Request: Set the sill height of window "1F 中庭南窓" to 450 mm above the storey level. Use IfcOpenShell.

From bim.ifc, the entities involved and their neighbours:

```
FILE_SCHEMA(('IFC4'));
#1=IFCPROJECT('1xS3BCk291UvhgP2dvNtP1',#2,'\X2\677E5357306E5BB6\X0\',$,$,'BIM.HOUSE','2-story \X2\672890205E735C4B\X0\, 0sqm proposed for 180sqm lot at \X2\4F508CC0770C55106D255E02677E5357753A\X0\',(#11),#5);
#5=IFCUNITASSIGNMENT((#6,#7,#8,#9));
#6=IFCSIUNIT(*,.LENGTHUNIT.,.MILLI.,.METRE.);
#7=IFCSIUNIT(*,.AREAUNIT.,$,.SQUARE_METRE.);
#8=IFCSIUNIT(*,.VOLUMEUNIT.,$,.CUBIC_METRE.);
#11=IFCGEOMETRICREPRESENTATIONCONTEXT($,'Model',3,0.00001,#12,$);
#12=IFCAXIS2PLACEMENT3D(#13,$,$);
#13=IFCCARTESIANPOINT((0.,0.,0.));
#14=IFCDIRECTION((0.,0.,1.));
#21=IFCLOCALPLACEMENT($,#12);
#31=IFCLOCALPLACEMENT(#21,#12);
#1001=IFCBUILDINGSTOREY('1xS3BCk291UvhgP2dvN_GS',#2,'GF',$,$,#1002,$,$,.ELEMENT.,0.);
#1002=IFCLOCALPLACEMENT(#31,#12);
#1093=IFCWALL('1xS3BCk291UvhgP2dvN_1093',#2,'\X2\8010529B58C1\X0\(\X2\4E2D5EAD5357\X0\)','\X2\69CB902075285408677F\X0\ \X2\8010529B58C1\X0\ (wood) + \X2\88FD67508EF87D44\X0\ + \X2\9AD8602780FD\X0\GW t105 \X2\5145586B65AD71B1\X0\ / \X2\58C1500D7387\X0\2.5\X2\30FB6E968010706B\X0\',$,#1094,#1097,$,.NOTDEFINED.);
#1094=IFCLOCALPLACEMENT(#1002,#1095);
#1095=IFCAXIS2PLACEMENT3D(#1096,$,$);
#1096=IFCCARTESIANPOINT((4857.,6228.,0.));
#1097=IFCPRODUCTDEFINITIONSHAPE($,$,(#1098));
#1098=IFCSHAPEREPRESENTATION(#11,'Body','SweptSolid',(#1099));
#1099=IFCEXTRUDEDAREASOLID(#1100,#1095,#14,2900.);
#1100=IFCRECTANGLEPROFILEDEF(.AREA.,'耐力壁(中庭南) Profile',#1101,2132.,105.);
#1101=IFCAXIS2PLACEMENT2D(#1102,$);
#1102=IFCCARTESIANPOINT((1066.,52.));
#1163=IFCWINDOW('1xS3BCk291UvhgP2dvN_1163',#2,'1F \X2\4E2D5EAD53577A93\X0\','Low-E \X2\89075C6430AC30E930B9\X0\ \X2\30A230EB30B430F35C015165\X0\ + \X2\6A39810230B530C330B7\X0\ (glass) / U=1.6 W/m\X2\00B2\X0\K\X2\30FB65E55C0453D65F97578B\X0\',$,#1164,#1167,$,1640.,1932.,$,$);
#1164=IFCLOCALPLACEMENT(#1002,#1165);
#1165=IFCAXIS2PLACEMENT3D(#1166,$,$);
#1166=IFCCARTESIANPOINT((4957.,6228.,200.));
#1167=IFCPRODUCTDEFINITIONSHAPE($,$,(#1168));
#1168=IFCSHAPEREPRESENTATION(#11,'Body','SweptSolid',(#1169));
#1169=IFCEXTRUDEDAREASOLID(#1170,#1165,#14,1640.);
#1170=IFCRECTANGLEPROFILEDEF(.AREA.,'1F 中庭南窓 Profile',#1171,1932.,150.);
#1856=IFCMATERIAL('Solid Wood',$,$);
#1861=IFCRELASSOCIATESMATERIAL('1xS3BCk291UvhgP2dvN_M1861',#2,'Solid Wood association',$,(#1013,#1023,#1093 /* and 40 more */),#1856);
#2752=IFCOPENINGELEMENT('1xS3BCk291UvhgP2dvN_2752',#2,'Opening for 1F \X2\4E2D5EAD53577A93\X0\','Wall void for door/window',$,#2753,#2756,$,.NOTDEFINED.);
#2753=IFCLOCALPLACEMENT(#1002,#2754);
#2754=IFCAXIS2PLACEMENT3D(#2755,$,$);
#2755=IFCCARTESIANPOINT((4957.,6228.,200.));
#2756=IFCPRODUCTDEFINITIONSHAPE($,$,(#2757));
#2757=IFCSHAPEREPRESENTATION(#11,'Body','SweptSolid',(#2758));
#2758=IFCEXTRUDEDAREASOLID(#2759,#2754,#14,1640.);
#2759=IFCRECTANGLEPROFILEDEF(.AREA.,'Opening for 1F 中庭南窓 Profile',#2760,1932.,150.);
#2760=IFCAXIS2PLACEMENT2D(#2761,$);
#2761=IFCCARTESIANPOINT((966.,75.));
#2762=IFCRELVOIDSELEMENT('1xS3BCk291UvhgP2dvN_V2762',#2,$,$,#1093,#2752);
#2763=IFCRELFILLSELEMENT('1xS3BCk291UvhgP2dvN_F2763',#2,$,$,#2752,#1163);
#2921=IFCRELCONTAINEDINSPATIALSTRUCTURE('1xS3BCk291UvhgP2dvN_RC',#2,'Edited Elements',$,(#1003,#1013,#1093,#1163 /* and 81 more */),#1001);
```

```python
import numpy as np
import ifcopenshell
import ifcopenshell.api.geometry
import ifcopenshell.geom
import ifcopenshell.util.element
import ifcopenshell.util.placement
import ifcopenshell.util.shape
import ifcopenshell.util.unit

model = ifcopenshell.open("bim.ifc")
unit_scale = ifcopenshell.util.unit.calculate_unit_scale(model)

window = model.by_guid("1xS3BCk291UvhgP2dvN_1163")
opening = window.FillsVoids[0].RelatingOpeningElement
storey = ifcopenshell.util.element.get_container(window, ifc_class="IfcBuildingStorey")
level = ifcopenshell.util.placement.get_local_placement(storey.ObjectPlacement)[2, 3]

# The opening's origin need not be at the sill, so measure its lowest point.
shape = ifcopenshell.geom.create_shape(ifcopenshell.geom.settings(), opening)
bottom = ifcopenshell.util.shape.get_shape_bottom_elevation(shape, shape.geometry) / unit_scale
dz = level + 450.0 - bottom

shift = np.array([0.0, 0.0, dz])
# The window is not placed relative to its opening, so move both.
for product in (opening, window):
    matrix = ifcopenshell.util.placement.get_local_placement(product.ObjectPlacement)
    matrix[:3, 3] += shift
    ifcopenshell.api.geometry.edit_object_placement(model, product=product, matrix=matrix, is_si=False)

print(f"moved by {dz * unit_scale:+.3f} m")

model.write("bim_rev.ifc")
```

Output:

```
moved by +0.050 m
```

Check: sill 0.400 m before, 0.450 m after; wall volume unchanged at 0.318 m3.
